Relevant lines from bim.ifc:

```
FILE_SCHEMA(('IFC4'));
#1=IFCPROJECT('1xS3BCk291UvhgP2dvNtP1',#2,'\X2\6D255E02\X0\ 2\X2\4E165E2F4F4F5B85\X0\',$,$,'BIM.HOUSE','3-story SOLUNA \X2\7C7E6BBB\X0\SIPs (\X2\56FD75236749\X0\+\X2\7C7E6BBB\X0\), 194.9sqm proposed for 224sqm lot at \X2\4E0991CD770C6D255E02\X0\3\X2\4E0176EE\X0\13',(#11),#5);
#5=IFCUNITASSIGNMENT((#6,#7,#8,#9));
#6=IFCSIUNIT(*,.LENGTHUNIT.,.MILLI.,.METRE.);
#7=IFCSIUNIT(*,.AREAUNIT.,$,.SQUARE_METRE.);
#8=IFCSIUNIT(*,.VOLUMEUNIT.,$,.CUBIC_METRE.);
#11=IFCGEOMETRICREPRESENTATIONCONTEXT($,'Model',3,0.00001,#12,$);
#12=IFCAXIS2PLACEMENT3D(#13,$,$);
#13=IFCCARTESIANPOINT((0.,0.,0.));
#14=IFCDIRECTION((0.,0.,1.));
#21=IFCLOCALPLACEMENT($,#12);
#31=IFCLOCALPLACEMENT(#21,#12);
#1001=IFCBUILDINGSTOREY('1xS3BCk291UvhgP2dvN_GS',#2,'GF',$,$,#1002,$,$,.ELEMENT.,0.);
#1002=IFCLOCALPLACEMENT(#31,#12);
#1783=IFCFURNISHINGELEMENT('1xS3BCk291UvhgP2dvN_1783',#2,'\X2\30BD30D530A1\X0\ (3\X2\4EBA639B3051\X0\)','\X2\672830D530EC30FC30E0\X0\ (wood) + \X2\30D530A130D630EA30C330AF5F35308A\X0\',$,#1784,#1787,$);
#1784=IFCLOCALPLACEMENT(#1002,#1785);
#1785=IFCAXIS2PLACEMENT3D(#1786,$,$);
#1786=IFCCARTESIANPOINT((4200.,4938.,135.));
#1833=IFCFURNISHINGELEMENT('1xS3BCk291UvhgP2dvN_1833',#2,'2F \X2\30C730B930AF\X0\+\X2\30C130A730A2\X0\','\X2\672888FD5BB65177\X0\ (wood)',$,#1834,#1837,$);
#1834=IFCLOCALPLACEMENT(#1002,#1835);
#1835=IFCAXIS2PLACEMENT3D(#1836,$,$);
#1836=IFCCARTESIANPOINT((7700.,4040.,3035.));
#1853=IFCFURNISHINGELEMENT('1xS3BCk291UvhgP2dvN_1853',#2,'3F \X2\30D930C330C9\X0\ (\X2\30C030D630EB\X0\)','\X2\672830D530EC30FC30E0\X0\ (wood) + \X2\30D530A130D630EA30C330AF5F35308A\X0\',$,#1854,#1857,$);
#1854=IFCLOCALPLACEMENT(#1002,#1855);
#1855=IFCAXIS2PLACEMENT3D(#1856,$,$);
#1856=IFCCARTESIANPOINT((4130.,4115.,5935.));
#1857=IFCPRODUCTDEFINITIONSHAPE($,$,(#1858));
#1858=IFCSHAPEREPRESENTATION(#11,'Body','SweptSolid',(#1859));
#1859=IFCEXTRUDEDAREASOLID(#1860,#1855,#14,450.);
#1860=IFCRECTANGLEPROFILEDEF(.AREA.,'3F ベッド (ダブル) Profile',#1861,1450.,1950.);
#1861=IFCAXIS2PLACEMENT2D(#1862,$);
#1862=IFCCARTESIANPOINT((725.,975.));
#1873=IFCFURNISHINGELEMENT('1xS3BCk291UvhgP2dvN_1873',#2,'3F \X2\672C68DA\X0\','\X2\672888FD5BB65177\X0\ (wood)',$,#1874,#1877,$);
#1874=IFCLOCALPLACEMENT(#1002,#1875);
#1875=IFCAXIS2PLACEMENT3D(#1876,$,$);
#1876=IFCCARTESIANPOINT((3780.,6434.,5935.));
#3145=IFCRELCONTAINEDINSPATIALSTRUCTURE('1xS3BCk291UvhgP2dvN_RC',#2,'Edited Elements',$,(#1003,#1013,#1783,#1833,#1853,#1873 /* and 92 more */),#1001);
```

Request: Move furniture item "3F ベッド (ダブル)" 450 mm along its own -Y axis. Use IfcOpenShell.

```python
import ifcopenshell
import ifcopenshell.api.geometry
import ifcopenshell.util.placement
import ifcopenshell.util.unit

model = ifcopenshell.open("bim.ifc")
unit_scale = ifcopenshell.util.unit.calculate_unit_scale(model)

item = model.by_guid("1xS3BCk291UvhgP2dvN_1853")
matrix = ifcopenshell.util.placement.get_local_placement(item.ObjectPlacement)
matrix[:3, 3] -= matrix[:3, 1] * 0.45 / unit_scale
ifcopenshell.api.geometry.edit_object_placement(model, product=item, matrix=matrix, is_si=False)

print(ifcopenshell.util.placement.get_local_placement(item.ObjectPlacement).round(3) + 0.0)

model.write("bim_updated.ifc")
```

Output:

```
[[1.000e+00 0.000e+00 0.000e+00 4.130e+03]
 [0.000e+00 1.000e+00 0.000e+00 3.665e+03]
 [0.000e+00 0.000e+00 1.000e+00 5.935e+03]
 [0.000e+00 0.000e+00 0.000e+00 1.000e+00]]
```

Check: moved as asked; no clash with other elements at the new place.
